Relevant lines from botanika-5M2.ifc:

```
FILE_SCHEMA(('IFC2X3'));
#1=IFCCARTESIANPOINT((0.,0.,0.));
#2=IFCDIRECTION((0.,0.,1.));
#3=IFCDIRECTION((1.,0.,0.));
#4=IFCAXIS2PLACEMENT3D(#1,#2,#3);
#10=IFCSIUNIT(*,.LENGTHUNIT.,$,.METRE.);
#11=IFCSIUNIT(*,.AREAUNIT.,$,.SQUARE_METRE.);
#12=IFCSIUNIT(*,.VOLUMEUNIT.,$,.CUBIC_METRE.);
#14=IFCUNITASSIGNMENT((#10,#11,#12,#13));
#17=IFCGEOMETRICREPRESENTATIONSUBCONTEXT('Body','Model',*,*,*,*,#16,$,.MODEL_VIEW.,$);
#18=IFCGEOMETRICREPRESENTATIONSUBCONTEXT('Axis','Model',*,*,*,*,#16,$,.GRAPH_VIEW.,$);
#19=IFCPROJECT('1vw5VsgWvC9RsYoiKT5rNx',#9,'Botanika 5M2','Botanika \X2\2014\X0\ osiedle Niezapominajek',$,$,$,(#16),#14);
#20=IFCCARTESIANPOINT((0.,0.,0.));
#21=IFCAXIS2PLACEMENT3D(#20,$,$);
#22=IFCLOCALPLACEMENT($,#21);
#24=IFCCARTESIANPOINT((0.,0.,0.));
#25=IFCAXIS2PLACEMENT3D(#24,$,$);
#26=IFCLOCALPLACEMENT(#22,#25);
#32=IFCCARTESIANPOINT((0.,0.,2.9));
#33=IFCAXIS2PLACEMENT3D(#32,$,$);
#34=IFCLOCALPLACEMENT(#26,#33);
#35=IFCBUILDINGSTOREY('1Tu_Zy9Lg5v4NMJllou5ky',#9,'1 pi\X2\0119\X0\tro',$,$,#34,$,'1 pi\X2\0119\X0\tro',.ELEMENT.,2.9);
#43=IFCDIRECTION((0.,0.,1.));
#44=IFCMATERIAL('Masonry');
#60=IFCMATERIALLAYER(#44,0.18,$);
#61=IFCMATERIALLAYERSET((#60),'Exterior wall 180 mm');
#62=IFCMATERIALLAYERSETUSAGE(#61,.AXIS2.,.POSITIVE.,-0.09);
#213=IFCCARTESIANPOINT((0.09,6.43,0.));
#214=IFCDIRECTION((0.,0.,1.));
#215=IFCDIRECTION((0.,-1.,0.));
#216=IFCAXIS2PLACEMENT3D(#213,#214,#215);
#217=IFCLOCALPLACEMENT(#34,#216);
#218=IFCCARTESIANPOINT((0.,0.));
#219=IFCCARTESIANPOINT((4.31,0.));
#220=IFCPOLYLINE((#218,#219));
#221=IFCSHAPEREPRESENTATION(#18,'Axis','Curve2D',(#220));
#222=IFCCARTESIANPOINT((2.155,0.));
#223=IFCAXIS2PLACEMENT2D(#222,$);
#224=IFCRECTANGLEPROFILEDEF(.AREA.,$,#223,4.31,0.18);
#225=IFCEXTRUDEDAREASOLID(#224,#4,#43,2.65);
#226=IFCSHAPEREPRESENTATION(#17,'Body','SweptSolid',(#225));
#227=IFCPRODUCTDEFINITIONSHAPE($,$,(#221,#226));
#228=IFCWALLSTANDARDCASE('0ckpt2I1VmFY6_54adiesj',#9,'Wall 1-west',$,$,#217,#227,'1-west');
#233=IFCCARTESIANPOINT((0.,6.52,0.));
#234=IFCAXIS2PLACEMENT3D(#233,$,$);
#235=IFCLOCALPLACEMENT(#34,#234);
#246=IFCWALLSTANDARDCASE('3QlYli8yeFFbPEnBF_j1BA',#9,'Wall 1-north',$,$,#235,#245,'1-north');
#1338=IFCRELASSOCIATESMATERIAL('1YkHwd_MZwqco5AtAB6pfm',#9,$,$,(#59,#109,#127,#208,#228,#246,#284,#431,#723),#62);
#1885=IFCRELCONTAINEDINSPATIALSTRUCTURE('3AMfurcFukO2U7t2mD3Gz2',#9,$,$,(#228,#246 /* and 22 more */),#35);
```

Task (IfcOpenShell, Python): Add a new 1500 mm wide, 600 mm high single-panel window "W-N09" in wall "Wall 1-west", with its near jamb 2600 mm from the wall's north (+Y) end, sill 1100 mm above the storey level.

```python
import numpy as np
import ifcopenshell
import ifcopenshell.api.feature
import ifcopenshell.api.geometry
import ifcopenshell.api.root
import ifcopenshell.api.spatial
import ifcopenshell.api.type
import ifcopenshell.geom
import ifcopenshell.util.element
import ifcopenshell.util.placement
import ifcopenshell.util.representation
import ifcopenshell.util.shape
import ifcopenshell.util.unit

model = ifcopenshell.open("botanika-5M2.ifc")
unit_scale = ifcopenshell.util.unit.calculate_unit_scale(model)
settings = ifcopenshell.geom.settings()


def volume(element):
    """Net volume in cubic metres, openings subtracted."""
    shape = ifcopenshell.geom.create_shape(settings, element)
    return ifcopenshell.util.shape.get_volume(shape.geometry)


wall = model.by_id(228)
storey = ifcopenshell.util.element.get_container(wall, ifc_class="IfcBuildingStorey")
context = ifcopenshell.util.representation.get_context(model, "Model", "Body", "MODEL_VIEW")
before = volume(wall)

width, height, from_end, sill = 1.5, 0.6, 2.6, 1.1  # metres

# The wall runs along its own X axis, and the end named is its -X end.
wall_shape = ifcopenshell.geom.create_shape(settings, wall)
x, y, z = ifcopenshell.util.shape.get_vertices(wall_shape.geometry).T
start = x.min() + from_end
face, thickness = float(y.min()), float(y.max() - y.min())
wall_matrix = ifcopenshell.util.placement.get_local_placement(wall.ObjectPlacement)
level = ifcopenshell.util.placement.get_local_placement(storey.ObjectPlacement)[2, 3]


def in_wall(x, y):
    """Placement at x, y metres in the wall's axes, at sill height."""
    matrix = wall_matrix.copy()
    matrix[:, 3] = wall_matrix @ np.array([x / unit_scale, y / unit_scale, 0.0, 1.0])
    matrix[2, 3] = level + sill / unit_scale
    return matrix


# Opening: a box that overshoots both wall faces by 50 mm.
opening = ifcopenshell.api.root.create_entity(model, ifc_class="IfcOpeningElement")
box = ifcopenshell.api.geometry.add_wall_representation(
    model, context=context, length=width, height=height, thickness=thickness + 0.1
)
ifcopenshell.api.geometry.assign_representation(model, product=opening, representation=box)
ifcopenshell.api.geometry.edit_object_placement(model, product=opening, matrix=in_wall(start, face - 0.05), is_si=False)
ifcopenshell.api.feature.add_feature(model, feature=opening, element=wall)

window = ifcopenshell.api.root.create_entity(model, ifc_class="IfcWindow", name="W-N09")
window.OverallWidth, window.OverallHeight = width / unit_scale, height / unit_scale
body = ifcopenshell.api.geometry.add_window_representation(
    model,
    context=context,
    overall_width=window.OverallWidth,
    overall_height=window.OverallHeight,
    partition_type="SINGLE_PANEL",
)
ifcopenshell.api.geometry.assign_representation(model, product=window, representation=body)
ifcopenshell.api.spatial.assign_container(model, products=[window], relating_structure=storey)
fills = ifcopenshell.api.feature.add_filling(model, opening=opening, element=window)
fills.OwnerHistory = window.OwnerHistory  # required in IFC2X3

# IFC2X3 keeps the operation on the window style.
style = ifcopenshell.api.root.create_entity(model, ifc_class="IfcWindowStyle", name="W-N09")
style.OperationType, style.ConstructionType = "SINGLE_PANEL", "NOTDEFINED"
style.ParameterTakesPrecedence = style.Sizeable = False
ifcopenshell.api.type.assign_type(model, related_objects=[window], relating_type=style)

# Centre the window in the wall's thickness.
ifcopenshell.api.geometry.edit_object_placement(model, product=window, matrix=in_wall(start, face), is_si=False)
window_shape = ifcopenshell.geom.create_shape(settings, window)
depth = ifcopenshell.util.shape.get_vertices(window_shape.geometry)[:, 1]
offset = face + thickness / 2 - (depth.min() + depth.max()) / 2
ifcopenshell.api.geometry.edit_object_placement(model, product=window, matrix=in_wall(start, offset), is_si=False)

after = volume(wall)

print(f"wall volume {before:.3f} -> {after:.3f} m3")

model.write("botanika-5M2-out.ifc")
```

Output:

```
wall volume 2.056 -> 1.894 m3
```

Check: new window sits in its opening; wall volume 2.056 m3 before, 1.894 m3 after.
